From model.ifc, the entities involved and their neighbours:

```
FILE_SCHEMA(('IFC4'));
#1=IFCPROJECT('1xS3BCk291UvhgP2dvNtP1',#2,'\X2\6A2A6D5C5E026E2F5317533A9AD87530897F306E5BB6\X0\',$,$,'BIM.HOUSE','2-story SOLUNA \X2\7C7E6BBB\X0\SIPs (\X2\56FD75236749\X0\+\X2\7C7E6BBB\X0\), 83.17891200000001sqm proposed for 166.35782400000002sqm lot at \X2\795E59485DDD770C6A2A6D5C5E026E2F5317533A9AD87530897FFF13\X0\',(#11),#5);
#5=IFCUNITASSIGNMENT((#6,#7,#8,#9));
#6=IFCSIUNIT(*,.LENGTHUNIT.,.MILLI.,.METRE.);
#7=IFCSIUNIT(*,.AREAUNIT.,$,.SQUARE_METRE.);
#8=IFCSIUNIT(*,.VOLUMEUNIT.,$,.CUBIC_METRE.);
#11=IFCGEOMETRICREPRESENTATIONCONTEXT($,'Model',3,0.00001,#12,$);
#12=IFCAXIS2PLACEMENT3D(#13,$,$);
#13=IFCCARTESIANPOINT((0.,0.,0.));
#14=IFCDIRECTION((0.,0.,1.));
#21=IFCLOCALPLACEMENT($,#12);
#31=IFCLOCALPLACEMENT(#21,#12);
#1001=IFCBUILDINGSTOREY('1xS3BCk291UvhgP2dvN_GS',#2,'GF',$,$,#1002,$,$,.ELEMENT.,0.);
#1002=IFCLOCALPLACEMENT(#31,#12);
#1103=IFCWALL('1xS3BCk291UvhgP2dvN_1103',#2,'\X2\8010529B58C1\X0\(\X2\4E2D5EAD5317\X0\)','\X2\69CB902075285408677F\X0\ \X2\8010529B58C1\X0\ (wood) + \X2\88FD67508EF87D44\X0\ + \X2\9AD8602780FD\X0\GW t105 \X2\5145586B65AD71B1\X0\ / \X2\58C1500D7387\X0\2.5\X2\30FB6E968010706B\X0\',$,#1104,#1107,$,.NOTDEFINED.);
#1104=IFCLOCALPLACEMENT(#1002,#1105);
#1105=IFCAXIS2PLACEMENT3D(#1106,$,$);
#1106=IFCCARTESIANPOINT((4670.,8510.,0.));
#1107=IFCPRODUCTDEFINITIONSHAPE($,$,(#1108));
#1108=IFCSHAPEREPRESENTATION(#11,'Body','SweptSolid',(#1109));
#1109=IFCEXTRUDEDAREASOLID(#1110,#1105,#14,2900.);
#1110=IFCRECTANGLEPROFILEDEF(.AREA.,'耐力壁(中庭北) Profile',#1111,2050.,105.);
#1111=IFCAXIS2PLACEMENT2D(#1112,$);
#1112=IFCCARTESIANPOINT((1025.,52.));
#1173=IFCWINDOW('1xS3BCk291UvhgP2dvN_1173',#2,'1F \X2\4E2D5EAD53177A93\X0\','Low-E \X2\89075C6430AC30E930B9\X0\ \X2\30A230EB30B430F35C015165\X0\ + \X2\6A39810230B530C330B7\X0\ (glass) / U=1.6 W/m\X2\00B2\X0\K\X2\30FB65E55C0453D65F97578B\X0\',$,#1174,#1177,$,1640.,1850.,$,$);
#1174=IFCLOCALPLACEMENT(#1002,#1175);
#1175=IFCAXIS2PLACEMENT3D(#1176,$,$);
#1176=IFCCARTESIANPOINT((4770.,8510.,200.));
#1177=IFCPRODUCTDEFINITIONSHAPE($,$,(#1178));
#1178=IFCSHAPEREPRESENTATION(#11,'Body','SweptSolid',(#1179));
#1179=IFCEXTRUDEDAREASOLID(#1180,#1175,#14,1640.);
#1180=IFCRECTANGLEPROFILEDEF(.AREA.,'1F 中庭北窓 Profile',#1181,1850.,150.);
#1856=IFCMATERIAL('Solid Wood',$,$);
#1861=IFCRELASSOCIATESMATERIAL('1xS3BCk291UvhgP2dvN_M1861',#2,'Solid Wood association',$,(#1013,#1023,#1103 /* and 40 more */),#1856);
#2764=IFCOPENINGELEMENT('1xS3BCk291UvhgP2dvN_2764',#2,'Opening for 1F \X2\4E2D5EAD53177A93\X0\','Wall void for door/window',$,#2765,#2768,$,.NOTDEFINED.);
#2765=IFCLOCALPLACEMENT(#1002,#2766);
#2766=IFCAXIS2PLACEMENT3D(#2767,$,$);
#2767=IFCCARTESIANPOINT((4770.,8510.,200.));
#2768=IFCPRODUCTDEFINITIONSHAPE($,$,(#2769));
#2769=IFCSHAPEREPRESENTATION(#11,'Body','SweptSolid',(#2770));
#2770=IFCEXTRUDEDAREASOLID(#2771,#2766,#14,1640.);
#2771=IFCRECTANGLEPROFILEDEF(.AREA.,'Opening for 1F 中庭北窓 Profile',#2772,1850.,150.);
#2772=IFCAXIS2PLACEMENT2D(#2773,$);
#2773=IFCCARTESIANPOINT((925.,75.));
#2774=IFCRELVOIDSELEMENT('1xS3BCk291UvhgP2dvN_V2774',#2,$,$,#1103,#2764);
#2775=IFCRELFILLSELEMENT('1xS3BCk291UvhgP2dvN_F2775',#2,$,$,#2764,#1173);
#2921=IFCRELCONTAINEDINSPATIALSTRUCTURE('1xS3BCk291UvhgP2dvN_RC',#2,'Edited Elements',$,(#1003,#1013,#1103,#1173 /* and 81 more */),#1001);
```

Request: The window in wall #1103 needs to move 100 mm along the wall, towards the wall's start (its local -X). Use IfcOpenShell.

```python
import ifcopenshell
import ifcopenshell.api.geometry
import ifcopenshell.util.placement
import ifcopenshell.util.unit

model = ifcopenshell.open("model.ifc")
unit_scale = ifcopenshell.util.unit.calculate_unit_scale(model)

window = model.by_guid("1xS3BCk291UvhgP2dvN_1173")
opening = window.FillsVoids[0].RelatingOpeningElement
wall = opening.VoidsElements[0].RelatingBuildingElement

wall_matrix = ifcopenshell.util.placement.get_local_placement(wall.ObjectPlacement)
shift = wall_matrix[:3, 0] * -0.1 / unit_scale
before = ifcopenshell.util.placement.get_local_placement(window.ObjectPlacement)[:3, 3].copy()

# The window is not placed relative to its opening, so move both.
for product in (opening, window):
    matrix = ifcopenshell.util.placement.get_local_placement(product.ObjectPlacement)
    matrix[:3, 3] += shift
    ifcopenshell.api.geometry.edit_object_placement(model, product=product, matrix=matrix, is_si=False)

after = ifcopenshell.util.placement.get_local_placement(window.ObjectPlacement)[:3, 3]
print("window moved by", (after - before).round(3) + 0.0)

model.write("model-out.ifc")
```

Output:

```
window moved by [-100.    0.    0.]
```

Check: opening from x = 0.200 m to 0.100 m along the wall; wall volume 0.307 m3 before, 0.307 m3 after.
